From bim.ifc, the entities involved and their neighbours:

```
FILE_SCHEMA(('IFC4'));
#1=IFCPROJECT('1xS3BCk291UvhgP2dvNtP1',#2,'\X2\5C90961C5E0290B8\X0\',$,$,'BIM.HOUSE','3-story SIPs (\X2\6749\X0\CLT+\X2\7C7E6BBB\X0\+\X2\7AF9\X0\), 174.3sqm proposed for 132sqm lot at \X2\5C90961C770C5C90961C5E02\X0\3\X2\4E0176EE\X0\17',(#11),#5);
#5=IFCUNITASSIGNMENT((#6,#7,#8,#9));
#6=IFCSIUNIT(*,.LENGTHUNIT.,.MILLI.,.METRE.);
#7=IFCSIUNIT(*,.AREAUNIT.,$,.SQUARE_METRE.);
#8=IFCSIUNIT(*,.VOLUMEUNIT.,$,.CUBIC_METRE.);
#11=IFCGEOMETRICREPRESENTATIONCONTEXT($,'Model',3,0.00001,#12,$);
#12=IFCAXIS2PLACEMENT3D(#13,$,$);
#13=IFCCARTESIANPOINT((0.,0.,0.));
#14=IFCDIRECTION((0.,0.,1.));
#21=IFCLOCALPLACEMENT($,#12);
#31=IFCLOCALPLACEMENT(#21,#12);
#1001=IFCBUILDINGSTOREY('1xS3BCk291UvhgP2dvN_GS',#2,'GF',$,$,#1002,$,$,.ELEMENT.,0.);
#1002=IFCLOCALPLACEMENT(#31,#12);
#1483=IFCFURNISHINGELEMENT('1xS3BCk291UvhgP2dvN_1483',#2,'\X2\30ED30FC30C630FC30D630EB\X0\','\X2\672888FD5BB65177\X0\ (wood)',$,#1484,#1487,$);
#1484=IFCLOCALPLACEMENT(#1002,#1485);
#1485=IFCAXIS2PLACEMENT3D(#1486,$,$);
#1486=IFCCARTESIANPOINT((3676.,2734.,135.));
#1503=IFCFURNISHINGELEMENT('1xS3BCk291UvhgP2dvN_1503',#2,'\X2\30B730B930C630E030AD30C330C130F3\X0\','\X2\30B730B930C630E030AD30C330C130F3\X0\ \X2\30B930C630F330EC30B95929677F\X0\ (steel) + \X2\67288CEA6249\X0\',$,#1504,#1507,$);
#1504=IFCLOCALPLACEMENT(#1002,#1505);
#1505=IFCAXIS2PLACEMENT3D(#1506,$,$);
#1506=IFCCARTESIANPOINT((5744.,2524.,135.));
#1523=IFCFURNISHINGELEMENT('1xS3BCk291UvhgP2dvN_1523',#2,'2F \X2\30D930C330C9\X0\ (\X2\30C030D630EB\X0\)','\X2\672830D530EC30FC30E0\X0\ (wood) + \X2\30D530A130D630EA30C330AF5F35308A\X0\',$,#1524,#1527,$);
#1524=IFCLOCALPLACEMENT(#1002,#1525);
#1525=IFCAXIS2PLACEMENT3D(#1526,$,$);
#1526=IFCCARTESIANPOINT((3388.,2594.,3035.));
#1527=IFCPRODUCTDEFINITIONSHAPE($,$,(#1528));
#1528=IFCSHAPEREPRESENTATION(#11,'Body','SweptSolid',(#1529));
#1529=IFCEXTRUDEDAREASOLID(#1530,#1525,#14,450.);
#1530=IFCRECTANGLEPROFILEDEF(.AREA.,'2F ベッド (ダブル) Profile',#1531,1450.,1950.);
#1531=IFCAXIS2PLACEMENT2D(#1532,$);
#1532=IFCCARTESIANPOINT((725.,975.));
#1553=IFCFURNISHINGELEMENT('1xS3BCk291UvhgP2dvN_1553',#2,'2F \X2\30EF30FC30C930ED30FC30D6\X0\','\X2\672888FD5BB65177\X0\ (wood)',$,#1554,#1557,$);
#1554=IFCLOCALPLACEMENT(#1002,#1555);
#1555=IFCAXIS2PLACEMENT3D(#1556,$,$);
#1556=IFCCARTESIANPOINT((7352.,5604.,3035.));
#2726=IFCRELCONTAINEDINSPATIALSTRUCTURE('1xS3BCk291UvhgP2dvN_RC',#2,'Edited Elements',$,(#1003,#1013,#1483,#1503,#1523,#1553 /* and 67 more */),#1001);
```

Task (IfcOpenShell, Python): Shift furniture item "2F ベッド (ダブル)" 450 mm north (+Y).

```python
import ifcopenshell
import ifcopenshell.api.geometry
import ifcopenshell.util.placement
import ifcopenshell.util.unit

model = ifcopenshell.open("bim.ifc")
unit_scale = ifcopenshell.util.unit.calculate_unit_scale(model)

item = model.by_guid("1xS3BCk291UvhgP2dvN_1523")
matrix = ifcopenshell.util.placement.get_local_placement(item.ObjectPlacement)
matrix[1, 3] += 0.45 / unit_scale
ifcopenshell.api.geometry.edit_object_placement(model, product=item, matrix=matrix, is_si=False)

print(ifcopenshell.util.placement.get_local_placement(item.ObjectPlacement).round(3) + 0.0)

model.write("bim_rev.ifc")
```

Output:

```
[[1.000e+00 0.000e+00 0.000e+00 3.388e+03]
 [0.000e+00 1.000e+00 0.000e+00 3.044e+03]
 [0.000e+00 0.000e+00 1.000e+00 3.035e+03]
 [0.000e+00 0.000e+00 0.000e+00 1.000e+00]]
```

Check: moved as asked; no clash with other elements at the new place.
